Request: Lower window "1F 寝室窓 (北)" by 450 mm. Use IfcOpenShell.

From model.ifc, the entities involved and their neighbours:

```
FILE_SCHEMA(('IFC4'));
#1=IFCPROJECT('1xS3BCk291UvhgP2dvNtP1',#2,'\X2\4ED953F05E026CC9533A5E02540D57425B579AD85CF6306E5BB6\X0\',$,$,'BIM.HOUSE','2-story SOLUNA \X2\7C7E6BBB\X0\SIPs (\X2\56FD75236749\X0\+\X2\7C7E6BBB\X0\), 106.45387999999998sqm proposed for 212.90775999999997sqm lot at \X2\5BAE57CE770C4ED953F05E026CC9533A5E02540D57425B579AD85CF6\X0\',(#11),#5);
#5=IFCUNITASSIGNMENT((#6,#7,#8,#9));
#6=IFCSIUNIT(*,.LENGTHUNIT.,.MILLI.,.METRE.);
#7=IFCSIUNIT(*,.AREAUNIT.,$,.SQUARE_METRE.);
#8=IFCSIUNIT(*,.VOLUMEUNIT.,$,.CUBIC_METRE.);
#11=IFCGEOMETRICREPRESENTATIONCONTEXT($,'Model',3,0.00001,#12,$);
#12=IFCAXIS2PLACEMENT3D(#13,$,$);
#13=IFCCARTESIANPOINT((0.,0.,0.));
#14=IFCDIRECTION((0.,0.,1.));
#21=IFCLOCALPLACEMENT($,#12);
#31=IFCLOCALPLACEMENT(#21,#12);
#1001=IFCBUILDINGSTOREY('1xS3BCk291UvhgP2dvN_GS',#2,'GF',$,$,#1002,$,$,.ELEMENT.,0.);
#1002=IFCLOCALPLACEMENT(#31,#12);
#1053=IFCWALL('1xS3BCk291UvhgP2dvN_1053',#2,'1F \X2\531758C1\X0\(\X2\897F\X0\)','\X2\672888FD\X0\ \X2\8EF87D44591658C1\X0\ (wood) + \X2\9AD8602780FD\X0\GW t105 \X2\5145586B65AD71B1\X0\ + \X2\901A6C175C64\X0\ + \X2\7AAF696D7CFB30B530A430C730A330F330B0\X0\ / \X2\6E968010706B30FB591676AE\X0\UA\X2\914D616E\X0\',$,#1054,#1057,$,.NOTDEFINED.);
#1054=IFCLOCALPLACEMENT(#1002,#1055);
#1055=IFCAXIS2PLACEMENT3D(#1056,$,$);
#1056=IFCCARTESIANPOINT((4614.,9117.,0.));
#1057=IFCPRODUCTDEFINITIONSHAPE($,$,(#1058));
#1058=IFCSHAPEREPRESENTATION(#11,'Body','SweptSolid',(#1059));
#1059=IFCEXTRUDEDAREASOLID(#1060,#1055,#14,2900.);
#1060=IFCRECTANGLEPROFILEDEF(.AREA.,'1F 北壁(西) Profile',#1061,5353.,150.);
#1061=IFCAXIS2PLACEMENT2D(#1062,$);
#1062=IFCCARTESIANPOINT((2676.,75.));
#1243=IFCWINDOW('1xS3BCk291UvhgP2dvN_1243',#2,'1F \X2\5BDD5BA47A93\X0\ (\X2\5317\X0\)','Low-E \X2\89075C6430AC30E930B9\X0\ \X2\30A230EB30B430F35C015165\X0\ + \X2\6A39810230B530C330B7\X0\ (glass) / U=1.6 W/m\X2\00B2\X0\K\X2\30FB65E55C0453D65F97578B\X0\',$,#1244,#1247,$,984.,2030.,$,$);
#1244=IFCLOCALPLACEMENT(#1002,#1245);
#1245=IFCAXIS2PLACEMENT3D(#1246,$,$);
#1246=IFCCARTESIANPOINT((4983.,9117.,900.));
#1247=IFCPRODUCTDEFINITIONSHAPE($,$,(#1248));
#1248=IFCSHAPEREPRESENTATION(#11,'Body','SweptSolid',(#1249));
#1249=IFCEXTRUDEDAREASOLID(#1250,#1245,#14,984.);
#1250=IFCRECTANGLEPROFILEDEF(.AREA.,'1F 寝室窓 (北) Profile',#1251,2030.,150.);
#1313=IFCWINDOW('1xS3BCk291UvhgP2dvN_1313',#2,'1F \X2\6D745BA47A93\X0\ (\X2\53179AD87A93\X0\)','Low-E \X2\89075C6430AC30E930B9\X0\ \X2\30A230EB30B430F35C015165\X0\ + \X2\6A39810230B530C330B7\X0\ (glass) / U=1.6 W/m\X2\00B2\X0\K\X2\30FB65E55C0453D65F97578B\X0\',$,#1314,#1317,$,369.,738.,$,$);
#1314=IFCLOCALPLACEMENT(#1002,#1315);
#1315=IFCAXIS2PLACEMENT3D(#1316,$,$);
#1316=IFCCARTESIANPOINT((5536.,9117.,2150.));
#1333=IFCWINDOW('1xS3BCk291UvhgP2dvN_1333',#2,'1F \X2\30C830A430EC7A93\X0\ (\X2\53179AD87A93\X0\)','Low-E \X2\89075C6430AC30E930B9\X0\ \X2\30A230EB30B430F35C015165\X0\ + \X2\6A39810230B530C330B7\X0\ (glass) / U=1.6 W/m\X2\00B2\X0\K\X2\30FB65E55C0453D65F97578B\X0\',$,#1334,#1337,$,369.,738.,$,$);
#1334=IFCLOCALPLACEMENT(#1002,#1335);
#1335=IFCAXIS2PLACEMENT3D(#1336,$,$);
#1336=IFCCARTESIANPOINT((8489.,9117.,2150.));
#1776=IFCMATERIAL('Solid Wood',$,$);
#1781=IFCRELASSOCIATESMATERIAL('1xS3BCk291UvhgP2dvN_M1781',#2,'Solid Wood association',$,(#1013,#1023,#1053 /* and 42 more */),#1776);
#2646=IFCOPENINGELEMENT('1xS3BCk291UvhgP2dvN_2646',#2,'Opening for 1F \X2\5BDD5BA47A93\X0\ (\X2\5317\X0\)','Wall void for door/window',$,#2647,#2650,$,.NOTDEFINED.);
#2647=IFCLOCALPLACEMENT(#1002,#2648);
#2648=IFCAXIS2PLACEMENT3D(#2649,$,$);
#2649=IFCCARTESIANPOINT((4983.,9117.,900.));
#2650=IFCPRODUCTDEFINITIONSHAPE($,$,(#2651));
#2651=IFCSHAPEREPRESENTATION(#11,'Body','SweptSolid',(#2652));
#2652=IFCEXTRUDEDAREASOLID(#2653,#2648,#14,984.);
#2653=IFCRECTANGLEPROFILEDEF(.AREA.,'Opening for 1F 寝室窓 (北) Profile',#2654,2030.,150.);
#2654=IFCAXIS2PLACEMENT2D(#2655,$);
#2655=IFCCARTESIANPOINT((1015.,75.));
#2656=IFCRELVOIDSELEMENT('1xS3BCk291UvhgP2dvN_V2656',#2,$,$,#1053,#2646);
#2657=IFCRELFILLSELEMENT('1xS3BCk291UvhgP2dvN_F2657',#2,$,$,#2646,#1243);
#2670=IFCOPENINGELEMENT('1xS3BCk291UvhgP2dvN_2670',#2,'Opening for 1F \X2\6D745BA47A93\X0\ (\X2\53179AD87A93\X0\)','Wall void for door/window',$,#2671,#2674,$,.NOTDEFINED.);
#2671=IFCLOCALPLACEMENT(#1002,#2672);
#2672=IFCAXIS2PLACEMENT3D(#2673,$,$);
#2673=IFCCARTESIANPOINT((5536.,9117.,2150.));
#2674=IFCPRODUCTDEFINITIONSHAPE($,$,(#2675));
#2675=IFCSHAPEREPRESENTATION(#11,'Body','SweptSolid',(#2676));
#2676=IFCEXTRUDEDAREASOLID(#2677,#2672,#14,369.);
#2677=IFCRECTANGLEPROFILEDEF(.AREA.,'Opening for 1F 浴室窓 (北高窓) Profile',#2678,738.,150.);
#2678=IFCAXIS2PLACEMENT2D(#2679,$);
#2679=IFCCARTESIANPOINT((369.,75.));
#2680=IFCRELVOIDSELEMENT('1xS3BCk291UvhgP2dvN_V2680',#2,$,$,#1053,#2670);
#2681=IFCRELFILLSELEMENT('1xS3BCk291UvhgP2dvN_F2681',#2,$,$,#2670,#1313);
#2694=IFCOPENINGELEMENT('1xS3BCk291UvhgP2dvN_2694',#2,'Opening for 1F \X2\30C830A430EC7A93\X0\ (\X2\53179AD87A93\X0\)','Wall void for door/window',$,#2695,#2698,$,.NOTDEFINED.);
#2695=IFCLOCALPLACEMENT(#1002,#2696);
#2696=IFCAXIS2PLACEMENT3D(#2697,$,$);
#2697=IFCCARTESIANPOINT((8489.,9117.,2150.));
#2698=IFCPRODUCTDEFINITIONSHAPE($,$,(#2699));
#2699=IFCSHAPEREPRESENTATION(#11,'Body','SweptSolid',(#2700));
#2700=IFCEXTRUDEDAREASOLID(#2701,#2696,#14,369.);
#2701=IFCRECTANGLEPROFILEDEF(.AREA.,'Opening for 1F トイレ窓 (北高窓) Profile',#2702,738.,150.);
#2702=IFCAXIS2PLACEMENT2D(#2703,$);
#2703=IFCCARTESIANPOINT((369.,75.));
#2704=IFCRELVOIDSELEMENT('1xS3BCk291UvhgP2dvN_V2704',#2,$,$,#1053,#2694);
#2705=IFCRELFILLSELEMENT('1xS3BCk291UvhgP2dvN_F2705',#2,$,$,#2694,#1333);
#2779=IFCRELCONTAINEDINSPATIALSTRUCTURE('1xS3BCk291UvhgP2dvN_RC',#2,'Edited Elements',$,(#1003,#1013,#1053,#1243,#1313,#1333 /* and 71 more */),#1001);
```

```python
import numpy as np
import ifcopenshell
import ifcopenshell.api.geometry
import ifcopenshell.util.placement
import ifcopenshell.util.unit

model = ifcopenshell.open("model.ifc")
unit_scale = ifcopenshell.util.unit.calculate_unit_scale(model)

window = model.by_guid("1xS3BCk291UvhgP2dvN_1243")
opening = window.FillsVoids[0].RelatingOpeningElement
dz = -450.0

shift = np.array([0.0, 0.0, dz])
# The window is not placed relative to its opening, so move both.
for product in (opening, window):
    matrix = ifcopenshell.util.placement.get_local_placement(product.ObjectPlacement)
    matrix[:3, 3] += shift
    ifcopenshell.api.geometry.edit_object_placement(model, product=product, matrix=matrix, is_si=False)

print(f"moved by {dz * unit_scale:+.3f} m")

model.write("model-out.ifc")
```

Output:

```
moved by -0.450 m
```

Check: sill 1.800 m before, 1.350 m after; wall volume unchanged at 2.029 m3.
